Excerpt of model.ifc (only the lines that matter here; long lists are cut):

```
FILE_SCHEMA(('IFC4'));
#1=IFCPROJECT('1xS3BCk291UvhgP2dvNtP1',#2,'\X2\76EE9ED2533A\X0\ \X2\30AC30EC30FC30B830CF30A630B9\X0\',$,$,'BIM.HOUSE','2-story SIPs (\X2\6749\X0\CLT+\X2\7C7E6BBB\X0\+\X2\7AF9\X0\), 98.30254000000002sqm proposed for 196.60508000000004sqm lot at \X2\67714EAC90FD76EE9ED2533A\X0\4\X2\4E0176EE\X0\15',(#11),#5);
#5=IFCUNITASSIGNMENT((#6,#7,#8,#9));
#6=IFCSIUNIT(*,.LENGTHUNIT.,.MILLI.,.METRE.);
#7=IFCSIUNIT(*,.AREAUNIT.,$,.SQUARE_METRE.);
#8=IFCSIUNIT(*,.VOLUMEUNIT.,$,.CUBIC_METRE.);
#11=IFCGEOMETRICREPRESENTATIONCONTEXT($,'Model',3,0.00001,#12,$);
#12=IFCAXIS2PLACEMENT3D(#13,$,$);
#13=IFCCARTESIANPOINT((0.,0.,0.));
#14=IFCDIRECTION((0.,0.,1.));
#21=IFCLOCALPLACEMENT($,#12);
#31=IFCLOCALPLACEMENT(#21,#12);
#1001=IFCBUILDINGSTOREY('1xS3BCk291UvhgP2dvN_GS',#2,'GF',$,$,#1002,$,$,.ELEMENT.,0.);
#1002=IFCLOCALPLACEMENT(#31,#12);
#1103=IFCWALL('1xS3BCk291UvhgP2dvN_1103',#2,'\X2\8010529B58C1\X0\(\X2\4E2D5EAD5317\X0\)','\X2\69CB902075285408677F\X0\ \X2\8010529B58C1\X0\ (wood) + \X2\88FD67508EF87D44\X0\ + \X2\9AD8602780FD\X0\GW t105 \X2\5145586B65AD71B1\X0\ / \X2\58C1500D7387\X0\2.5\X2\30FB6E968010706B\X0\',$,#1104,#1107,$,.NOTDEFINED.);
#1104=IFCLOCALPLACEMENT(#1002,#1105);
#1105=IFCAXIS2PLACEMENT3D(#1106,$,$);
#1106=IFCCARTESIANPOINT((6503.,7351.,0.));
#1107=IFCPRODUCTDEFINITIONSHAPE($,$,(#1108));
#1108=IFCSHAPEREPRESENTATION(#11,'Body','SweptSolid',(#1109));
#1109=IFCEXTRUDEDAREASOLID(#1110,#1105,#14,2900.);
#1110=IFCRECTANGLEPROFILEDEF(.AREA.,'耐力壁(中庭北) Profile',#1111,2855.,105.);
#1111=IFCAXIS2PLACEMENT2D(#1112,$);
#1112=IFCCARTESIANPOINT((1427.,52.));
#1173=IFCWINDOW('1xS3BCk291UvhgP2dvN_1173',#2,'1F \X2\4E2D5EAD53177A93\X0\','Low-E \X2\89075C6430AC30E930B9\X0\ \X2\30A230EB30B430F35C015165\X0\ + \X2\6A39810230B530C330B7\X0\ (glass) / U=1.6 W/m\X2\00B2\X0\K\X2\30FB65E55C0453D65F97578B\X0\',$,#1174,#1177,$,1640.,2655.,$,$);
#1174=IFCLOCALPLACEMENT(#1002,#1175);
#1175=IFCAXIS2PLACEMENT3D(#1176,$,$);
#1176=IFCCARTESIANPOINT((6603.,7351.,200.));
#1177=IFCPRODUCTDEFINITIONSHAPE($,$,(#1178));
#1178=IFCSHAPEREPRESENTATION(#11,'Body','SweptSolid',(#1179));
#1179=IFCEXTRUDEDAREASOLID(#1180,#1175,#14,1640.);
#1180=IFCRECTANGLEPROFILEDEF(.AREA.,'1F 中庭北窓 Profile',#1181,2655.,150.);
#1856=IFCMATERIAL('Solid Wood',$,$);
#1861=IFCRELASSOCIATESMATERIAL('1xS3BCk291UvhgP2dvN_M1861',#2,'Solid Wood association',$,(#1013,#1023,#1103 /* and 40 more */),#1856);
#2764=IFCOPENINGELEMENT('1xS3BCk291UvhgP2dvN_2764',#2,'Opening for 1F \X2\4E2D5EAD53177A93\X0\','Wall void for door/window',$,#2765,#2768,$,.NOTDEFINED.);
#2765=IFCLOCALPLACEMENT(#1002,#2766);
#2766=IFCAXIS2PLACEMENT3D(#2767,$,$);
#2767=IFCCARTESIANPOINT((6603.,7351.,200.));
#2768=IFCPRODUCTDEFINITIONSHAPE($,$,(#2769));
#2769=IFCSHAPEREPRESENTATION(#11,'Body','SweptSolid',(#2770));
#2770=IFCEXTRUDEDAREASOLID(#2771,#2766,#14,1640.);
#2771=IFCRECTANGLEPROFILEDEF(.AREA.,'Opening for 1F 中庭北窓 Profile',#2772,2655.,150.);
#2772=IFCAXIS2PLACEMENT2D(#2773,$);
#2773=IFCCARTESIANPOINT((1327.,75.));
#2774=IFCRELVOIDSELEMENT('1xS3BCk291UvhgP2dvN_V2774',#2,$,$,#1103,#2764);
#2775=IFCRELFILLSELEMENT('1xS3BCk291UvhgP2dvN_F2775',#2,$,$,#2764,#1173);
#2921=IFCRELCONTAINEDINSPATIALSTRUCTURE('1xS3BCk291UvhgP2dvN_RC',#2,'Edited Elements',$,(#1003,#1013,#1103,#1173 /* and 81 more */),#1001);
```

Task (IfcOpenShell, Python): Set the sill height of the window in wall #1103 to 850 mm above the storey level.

```python
import numpy as np
import ifcopenshell
import ifcopenshell.api.geometry
import ifcopenshell.geom
import ifcopenshell.util.element
import ifcopenshell.util.placement
import ifcopenshell.util.shape
import ifcopenshell.util.unit

model = ifcopenshell.open("model.ifc")
unit_scale = ifcopenshell.util.unit.calculate_unit_scale(model)

window = model.by_guid("1xS3BCk291UvhgP2dvN_1173")
opening = window.FillsVoids[0].RelatingOpeningElement
storey = ifcopenshell.util.element.get_container(window, ifc_class="IfcBuildingStorey")
level = ifcopenshell.util.placement.get_local_placement(storey.ObjectPlacement)[2, 3]

# The opening's origin need not be at the sill, so measure its lowest point.
shape = ifcopenshell.geom.create_shape(ifcopenshell.geom.settings(), opening)
bottom = ifcopenshell.util.shape.get_shape_bottom_elevation(shape, shape.geometry) / unit_scale
dz = level + 0.85 / unit_scale - bottom

shift = np.array([0.0, 0.0, dz])
# The window is not placed relative to its opening, so move both.
for product in (opening, window):
    matrix = ifcopenshell.util.placement.get_local_placement(product.ObjectPlacement)
    matrix[:3, 3] += shift
    ifcopenshell.api.geometry.edit_object_placement(model, product=product, matrix=matrix, is_si=False)

print(f"moved by {dz * unit_scale:+.3f} m")

model.write("model_edited.ifc")
```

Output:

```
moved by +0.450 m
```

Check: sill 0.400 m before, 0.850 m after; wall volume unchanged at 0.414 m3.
